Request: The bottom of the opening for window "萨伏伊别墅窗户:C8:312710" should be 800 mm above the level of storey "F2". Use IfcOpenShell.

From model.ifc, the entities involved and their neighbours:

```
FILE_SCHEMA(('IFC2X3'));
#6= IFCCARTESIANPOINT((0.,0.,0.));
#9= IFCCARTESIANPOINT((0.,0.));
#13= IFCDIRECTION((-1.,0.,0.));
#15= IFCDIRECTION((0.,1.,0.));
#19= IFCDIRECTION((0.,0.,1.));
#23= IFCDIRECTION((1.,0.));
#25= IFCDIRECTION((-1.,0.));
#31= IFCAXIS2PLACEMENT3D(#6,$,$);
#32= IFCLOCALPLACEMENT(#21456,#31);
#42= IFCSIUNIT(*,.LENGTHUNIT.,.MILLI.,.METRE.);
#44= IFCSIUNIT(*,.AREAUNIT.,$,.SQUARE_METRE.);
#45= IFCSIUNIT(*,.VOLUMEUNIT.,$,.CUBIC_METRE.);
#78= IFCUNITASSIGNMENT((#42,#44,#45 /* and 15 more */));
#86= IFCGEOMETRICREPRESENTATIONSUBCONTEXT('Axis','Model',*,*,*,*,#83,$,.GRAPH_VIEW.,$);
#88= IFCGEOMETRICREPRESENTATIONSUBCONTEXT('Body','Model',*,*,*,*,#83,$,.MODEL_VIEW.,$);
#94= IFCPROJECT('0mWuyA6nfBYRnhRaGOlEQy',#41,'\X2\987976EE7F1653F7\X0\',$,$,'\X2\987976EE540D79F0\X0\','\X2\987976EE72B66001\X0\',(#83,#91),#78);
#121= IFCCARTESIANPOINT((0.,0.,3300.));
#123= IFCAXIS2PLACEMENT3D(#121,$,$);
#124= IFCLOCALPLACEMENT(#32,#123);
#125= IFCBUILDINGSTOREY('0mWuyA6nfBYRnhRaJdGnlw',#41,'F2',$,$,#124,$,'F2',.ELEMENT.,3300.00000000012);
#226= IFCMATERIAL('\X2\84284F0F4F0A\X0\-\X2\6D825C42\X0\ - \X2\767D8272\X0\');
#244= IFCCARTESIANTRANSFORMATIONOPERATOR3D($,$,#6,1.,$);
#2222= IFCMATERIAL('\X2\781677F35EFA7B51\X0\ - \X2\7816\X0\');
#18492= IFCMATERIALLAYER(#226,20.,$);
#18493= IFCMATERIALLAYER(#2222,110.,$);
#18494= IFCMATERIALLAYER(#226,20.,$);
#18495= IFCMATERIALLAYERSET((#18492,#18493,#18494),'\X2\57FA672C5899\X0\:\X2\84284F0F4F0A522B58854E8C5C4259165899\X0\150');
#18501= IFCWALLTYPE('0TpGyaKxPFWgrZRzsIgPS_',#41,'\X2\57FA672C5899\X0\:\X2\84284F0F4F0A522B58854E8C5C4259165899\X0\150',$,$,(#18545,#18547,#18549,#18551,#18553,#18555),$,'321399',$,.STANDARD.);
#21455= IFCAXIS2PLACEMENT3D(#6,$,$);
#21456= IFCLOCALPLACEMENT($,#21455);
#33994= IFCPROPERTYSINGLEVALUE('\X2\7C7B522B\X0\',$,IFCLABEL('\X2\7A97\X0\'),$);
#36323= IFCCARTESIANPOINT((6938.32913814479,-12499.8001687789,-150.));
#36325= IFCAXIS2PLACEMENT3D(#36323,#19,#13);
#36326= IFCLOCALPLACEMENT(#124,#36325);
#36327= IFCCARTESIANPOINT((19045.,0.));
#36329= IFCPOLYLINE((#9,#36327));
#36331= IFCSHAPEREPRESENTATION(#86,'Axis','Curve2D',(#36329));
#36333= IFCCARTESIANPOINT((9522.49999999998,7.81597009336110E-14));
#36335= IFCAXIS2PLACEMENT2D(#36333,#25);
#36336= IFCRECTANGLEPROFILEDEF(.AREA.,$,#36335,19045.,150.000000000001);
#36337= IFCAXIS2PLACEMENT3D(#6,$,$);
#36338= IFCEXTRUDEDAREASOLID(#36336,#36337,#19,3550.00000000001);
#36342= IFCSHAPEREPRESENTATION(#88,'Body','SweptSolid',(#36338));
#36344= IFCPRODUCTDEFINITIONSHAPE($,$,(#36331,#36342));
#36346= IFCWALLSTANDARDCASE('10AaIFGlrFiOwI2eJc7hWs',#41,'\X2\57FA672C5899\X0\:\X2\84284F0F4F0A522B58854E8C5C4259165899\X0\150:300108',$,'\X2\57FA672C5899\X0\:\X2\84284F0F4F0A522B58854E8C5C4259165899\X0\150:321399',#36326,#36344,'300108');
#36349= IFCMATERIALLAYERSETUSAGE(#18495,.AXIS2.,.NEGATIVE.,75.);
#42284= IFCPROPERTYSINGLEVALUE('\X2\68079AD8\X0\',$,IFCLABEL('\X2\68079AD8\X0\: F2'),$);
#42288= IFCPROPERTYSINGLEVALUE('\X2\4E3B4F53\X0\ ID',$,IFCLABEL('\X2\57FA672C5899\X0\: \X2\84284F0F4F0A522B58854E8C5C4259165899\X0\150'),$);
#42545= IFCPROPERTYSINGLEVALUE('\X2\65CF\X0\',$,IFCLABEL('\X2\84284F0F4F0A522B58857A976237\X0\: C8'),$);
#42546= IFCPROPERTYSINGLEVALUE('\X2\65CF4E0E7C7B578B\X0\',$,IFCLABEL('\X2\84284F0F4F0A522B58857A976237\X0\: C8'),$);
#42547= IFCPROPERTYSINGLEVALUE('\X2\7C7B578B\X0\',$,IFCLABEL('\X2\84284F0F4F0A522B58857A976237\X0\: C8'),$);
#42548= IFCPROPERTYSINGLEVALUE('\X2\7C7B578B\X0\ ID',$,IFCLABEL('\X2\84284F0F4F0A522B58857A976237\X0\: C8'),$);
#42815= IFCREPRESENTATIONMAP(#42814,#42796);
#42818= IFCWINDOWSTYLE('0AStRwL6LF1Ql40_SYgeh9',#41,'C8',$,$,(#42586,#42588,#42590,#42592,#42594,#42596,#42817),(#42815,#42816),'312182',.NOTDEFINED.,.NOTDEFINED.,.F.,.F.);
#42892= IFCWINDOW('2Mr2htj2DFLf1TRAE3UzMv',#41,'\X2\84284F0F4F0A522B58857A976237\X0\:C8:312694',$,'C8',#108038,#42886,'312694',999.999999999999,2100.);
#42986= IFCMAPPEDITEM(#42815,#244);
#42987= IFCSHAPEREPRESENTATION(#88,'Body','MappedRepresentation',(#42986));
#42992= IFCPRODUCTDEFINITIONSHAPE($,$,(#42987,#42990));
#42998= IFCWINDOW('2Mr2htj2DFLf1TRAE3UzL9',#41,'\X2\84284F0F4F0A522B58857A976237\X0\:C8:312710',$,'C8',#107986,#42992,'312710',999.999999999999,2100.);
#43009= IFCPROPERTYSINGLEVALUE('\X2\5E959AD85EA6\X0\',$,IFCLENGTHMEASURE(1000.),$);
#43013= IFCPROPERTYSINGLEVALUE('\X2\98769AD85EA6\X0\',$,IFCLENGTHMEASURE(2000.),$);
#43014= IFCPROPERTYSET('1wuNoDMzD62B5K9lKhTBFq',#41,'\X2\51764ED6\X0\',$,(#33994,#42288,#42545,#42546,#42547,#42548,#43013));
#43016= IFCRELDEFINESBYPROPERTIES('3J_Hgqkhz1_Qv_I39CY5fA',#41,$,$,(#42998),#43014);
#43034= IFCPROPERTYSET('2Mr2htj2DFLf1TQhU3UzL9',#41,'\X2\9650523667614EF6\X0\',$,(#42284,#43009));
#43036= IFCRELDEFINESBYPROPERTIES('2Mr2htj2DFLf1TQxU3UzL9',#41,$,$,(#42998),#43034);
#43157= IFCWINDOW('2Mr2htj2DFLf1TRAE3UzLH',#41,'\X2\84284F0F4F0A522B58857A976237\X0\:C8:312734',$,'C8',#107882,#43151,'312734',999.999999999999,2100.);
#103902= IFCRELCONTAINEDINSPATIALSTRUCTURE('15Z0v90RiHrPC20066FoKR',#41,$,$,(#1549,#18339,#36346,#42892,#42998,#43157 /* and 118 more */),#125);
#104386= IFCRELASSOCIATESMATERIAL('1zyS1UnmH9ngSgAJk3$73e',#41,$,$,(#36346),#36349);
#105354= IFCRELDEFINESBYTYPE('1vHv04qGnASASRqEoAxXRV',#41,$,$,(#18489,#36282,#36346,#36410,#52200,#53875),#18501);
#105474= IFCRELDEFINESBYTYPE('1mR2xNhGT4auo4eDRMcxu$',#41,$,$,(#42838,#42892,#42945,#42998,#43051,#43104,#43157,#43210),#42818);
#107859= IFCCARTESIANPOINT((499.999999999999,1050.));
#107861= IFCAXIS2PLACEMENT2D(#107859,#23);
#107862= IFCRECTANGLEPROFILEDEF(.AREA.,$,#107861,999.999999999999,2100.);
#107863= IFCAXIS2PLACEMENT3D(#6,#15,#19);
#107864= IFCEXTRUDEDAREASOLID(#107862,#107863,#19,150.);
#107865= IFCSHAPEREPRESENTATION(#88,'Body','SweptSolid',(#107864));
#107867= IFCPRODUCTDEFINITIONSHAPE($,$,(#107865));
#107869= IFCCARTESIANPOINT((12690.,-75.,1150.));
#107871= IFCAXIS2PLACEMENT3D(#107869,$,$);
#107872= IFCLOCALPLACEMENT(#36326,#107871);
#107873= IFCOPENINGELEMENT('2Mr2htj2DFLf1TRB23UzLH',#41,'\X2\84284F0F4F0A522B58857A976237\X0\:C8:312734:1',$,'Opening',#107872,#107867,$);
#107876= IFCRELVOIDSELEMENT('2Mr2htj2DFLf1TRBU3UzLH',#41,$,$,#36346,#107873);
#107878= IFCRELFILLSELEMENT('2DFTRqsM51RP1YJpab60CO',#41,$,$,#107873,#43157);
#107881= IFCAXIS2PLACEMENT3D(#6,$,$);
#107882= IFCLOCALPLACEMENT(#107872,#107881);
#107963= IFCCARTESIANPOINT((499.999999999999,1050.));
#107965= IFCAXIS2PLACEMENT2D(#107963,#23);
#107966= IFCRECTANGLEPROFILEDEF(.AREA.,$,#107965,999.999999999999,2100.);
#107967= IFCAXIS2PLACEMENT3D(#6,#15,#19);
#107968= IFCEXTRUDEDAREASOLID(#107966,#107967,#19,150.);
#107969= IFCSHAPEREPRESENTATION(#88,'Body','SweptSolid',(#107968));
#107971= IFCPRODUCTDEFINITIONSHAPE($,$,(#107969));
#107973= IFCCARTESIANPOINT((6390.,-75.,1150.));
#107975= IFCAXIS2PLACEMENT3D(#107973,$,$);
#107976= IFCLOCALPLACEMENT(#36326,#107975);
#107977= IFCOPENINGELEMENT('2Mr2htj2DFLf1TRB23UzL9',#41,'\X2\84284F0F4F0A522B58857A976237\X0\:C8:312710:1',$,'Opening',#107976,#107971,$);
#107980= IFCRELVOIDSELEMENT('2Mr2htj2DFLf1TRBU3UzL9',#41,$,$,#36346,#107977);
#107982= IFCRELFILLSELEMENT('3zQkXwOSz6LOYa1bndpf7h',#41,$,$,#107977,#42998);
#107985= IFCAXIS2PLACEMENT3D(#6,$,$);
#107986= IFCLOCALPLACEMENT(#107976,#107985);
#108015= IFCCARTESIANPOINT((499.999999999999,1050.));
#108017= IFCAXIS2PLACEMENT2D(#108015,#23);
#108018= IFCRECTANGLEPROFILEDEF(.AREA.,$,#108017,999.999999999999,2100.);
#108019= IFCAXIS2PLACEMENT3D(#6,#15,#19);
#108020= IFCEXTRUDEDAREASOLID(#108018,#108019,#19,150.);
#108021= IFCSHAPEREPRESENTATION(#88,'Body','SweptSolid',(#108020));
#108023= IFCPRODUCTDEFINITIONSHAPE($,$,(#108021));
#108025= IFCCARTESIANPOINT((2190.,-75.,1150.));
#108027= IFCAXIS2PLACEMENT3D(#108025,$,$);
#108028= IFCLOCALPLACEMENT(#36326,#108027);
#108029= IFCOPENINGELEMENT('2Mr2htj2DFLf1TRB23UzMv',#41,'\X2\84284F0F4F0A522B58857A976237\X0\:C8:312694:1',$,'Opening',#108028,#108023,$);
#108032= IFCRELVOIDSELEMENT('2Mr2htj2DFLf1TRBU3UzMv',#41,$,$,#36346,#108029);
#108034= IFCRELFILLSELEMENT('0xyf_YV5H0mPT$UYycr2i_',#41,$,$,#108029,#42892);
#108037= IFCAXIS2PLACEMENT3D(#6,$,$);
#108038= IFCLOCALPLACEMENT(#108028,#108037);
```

```python
import numpy as np
import ifcopenshell
import ifcopenshell.api.geometry
import ifcopenshell.api.pset
import ifcopenshell.geom
import ifcopenshell.util.element
import ifcopenshell.util.placement
import ifcopenshell.util.shape
import ifcopenshell.util.unit

model = ifcopenshell.open("model.ifc")
unit_scale = ifcopenshell.util.unit.calculate_unit_scale(model)

window = model.by_id(42998)
opening = window.FillsVoids[0].RelatingOpeningElement
storey = ifcopenshell.util.element.get_container(window, ifc_class="IfcBuildingStorey")
level = ifcopenshell.util.placement.get_local_placement(storey.ObjectPlacement)[2, 3]

# The opening's origin need not be at the sill, so measure its lowest point.
shape = ifcopenshell.geom.create_shape(ifcopenshell.geom.settings(), opening)
bottom = ifcopenshell.util.shape.get_shape_bottom_elevation(shape, shape.geometry) / unit_scale
dz = level + 800.0 - bottom

shift = np.array([0.0, 0.0, dz])
# The window is placed relative to its opening, so it follows when the opening moves.
matrix = ifcopenshell.util.placement.get_local_placement(opening.ObjectPlacement)
matrix[:3, 3] += shift
ifcopenshell.api.geometry.edit_object_placement(
    model, product=opening, matrix=matrix, is_si=False, should_transform_children=True
)

# Keep the stored heights in step.
pset = model.by_id(ifcopenshell.util.element.get_pset(window, "其他", should_inherit=False)["id"])
ifcopenshell.api.pset.edit_pset(model, pset=pset, properties={
    "顶高度": model.create_entity("IfcLengthMeasure", ifcopenshell.util.element.get_pset(window, "其他", "顶高度") + dz),
})
pset = model.by_id(ifcopenshell.util.element.get_pset(window, "限制条件", should_inherit=False)["id"])
ifcopenshell.api.pset.edit_pset(model, pset=pset, properties={
    "底高度": model.create_entity("IfcLengthMeasure", ifcopenshell.util.element.get_pset(window, "限制条件", "底高度") + dz),
})

print(f"moved by {dz * unit_scale:+.3f} m")

model.write("model_edited.ifc")
```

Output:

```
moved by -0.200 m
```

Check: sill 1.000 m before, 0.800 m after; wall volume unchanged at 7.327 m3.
